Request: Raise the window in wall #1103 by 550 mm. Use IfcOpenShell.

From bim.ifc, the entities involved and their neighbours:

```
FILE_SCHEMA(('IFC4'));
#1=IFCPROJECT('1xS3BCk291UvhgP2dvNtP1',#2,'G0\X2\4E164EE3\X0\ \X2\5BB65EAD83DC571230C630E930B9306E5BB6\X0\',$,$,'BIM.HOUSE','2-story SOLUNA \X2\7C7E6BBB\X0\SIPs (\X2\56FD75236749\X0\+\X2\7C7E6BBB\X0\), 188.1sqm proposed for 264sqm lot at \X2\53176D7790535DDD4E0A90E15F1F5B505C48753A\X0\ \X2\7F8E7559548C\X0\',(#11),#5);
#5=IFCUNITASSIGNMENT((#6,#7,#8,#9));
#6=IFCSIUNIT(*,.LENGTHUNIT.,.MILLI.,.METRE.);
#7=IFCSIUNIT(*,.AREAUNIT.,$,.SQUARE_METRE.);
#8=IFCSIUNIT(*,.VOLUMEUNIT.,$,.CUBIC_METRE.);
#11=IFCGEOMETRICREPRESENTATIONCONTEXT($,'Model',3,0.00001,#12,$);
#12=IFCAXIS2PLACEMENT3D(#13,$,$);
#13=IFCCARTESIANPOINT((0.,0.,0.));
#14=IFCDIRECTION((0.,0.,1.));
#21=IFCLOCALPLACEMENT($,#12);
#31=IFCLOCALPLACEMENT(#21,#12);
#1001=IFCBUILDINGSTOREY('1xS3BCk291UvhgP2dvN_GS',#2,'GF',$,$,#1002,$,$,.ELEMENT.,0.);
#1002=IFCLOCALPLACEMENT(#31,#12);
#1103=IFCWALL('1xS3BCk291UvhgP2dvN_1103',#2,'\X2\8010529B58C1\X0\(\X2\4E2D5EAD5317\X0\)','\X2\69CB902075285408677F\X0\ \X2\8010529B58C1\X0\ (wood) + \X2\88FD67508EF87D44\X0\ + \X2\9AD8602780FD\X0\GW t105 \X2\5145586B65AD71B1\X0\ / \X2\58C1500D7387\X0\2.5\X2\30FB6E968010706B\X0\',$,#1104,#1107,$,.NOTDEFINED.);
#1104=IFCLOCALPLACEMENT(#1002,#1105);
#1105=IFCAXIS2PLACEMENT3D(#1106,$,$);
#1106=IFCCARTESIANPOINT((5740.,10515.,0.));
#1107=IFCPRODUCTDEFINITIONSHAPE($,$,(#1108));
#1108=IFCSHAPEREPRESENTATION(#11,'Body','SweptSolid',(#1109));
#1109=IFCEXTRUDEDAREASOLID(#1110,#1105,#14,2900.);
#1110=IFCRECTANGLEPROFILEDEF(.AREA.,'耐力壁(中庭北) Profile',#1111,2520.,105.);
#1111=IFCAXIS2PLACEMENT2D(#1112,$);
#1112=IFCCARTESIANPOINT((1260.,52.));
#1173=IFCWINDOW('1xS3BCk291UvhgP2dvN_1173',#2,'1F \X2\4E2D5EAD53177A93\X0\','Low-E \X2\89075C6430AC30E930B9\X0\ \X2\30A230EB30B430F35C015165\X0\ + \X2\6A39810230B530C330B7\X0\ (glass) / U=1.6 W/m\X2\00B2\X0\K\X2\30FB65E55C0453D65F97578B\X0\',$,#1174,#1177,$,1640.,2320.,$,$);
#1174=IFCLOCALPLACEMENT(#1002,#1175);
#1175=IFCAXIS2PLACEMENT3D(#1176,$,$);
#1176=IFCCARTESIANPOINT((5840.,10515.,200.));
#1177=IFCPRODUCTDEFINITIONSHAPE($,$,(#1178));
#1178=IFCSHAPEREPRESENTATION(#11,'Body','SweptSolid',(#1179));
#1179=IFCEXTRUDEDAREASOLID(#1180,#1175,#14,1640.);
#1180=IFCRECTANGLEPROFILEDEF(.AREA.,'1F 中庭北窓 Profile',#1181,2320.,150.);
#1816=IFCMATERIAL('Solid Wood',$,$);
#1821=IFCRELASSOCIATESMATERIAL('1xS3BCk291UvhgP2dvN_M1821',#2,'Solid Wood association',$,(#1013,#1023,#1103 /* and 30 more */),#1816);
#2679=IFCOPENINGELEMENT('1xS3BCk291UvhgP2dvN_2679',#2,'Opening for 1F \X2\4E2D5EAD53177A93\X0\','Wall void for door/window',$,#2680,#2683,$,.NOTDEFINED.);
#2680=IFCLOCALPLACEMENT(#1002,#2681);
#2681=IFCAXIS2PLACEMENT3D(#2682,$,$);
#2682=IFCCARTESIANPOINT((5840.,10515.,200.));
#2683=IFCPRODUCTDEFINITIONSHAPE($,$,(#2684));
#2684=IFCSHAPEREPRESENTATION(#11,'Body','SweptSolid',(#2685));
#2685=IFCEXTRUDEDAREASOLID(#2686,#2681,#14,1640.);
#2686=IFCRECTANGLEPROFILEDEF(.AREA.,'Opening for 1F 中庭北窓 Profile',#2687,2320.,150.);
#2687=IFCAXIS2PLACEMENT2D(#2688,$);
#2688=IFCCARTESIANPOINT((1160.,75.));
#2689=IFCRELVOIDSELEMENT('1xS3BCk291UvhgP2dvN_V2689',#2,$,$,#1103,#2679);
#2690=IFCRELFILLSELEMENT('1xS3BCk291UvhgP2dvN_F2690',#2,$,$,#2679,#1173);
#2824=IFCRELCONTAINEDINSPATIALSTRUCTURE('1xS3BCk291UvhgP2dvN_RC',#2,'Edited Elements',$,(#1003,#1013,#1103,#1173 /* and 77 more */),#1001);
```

```python
import numpy as np
import ifcopenshell
import ifcopenshell.api.geometry
import ifcopenshell.util.placement
import ifcopenshell.util.unit

model = ifcopenshell.open("bim.ifc")
unit_scale = ifcopenshell.util.unit.calculate_unit_scale(model)

window = model.by_guid("1xS3BCk291UvhgP2dvN_1173")
opening = window.FillsVoids[0].RelatingOpeningElement
dz = 550.0

shift = np.array([0.0, 0.0, dz])
# The window is not placed relative to its opening, so move both.
for product in (opening, window):
    matrix = ifcopenshell.util.placement.get_local_placement(product.ObjectPlacement)
    matrix[:3, 3] += shift
    ifcopenshell.api.geometry.edit_object_placement(model, product=product, matrix=matrix, is_si=False)

print(f"moved by {dz * unit_scale:+.3f} m")

model.write("bim_edited.ifc")
```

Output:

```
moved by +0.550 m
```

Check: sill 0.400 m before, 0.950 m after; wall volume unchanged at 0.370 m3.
